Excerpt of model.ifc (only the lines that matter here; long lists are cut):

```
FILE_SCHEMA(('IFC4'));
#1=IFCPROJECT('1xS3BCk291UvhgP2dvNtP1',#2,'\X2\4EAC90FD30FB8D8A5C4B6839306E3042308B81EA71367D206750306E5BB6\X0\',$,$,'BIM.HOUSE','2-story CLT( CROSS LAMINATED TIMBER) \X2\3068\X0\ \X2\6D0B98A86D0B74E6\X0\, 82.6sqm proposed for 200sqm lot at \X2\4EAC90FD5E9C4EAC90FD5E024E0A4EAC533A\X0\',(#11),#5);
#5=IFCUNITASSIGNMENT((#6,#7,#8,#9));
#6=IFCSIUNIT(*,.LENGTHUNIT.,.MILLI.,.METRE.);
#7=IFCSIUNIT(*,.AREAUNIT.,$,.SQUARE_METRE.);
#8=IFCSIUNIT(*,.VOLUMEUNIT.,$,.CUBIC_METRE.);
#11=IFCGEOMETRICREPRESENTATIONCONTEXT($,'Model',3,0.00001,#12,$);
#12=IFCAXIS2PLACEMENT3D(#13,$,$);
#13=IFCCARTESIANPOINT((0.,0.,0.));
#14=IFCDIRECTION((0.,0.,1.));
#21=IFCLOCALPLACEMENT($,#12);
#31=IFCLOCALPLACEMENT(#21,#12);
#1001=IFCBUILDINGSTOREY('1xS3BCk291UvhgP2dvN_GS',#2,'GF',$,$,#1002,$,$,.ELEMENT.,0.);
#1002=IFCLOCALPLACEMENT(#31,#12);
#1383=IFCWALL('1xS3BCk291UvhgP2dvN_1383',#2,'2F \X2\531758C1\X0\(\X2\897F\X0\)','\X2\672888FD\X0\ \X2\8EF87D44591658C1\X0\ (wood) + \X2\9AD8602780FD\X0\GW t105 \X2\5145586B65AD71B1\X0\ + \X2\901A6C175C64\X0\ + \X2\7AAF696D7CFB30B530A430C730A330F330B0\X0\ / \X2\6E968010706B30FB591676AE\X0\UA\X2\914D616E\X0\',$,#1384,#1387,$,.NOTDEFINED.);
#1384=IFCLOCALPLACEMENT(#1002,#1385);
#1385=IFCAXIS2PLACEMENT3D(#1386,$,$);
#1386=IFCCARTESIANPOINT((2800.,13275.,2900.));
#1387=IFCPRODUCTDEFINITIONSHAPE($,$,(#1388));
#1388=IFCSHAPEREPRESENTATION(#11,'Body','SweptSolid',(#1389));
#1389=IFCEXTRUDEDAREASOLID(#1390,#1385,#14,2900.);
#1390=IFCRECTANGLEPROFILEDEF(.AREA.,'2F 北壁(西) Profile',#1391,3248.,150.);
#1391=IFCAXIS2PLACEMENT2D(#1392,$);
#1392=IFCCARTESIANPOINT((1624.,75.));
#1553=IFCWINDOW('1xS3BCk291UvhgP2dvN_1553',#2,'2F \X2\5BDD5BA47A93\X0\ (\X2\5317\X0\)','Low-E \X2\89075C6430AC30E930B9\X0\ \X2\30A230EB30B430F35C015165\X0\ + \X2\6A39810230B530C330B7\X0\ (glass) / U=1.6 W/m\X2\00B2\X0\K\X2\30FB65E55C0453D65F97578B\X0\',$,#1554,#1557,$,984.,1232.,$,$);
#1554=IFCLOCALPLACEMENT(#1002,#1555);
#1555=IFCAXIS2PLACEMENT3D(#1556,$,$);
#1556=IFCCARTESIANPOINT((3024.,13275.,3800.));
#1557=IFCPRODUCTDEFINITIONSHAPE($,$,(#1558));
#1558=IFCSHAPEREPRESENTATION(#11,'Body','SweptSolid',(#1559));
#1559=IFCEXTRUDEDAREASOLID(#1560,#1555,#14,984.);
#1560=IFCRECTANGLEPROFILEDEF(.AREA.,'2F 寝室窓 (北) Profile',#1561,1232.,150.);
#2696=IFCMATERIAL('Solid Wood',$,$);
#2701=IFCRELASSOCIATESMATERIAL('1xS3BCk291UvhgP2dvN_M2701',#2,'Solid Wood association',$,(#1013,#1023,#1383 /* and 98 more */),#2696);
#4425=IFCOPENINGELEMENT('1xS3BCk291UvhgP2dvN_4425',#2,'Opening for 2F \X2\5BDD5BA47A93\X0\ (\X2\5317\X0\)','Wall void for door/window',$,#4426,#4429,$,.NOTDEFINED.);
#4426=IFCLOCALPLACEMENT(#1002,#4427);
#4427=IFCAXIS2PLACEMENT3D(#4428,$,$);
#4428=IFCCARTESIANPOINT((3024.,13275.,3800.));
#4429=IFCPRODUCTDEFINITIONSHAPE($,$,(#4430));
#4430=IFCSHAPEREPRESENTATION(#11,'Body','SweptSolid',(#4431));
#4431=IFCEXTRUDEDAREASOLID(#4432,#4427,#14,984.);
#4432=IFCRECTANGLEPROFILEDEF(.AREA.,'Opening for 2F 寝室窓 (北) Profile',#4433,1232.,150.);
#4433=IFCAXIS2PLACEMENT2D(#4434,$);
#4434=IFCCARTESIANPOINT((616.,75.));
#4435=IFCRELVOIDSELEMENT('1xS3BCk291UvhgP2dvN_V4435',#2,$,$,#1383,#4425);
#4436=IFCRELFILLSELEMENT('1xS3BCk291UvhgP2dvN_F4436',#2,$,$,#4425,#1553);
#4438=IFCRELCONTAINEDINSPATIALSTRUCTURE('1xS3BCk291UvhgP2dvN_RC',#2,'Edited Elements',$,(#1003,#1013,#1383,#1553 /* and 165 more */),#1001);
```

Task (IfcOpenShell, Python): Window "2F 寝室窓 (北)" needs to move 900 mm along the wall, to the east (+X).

```python
import ifcopenshell
import ifcopenshell.api.geometry
import ifcopenshell.util.placement

model = ifcopenshell.open("model.ifc")

window = model.by_id(1553)
opening = window.FillsVoids[0].RelatingOpeningElement
wall = opening.VoidsElements[0].RelatingBuildingElement

wall_matrix = ifcopenshell.util.placement.get_local_placement(wall.ObjectPlacement)
shift = wall_matrix[:3, 0] * 900.0
before = ifcopenshell.util.placement.get_local_placement(window.ObjectPlacement)[:3, 3].copy()

# The window is not placed relative to its opening, so move both.
for product in (opening, window):
    matrix = ifcopenshell.util.placement.get_local_placement(product.ObjectPlacement)
    matrix[:3, 3] += shift
    ifcopenshell.api.geometry.edit_object_placement(model, product=product, matrix=matrix, is_si=False)

after = ifcopenshell.util.placement.get_local_placement(window.ObjectPlacement)[:3, 3]
print("window moved by", (after - before).round(3) + 0.0)

model.write("model_updated.ifc")
```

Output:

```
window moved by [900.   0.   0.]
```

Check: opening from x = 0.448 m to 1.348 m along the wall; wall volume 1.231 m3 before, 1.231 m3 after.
